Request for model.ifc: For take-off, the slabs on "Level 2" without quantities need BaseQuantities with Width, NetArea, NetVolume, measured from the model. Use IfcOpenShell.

First a look at what the model holds.

```python
import ifcopenshell
import ifcopenshell.util.element
import ifcopenshell.util.unit

model = ifcopenshell.open("model.ifc")
print(model.schema)
for unit_type in ("LENGTHUNIT", "AREAUNIT", "VOLUMEUNIT"):
    print(unit_type, ifcopenshell.util.unit.calculate_unit_scale(model, unit_type))
storey = next(s for s in model.by_type("IfcBuildingStorey") if s.Name == "Level 2")
slabs = [e for e in ifcopenshell.util.element.get_decomposition(storey) if e.is_a("IfcSlab")]
for e in sorted(slabs, key=lambda e: e.id()):
    print(e.id(), e.is_a(), e.Name, list(ifcopenshell.util.element.get_psets(e, qtos_only=True)), sep=" | ")
```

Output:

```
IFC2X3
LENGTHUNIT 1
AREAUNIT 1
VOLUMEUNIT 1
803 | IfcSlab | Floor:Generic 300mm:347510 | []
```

```python
import ifcopenshell
import ifcopenshell.api.pset
import ifcopenshell.geom
import ifcopenshell.util.element
import ifcopenshell.util.shape
import ifcopenshell.util.unit

model = ifcopenshell.open("model.ifc")
unit_scale = ifcopenshell.util.unit.calculate_unit_scale(model)
area_scale = ifcopenshell.util.unit.calculate_unit_scale(model, "AREAUNIT")
volume_scale = ifcopenshell.util.unit.calculate_unit_scale(model, "VOLUMEUNIT")
settings = ifcopenshell.geom.settings()

storey = next(s for s in model.by_type("IfcBuildingStorey") if s.Name == "Level 2")
slabs = [e for e in ifcopenshell.util.element.get_decomposition(storey) if e.is_a("IfcSlab")]

for e in sorted(slabs, key=lambda e: e.id()):
    if ifcopenshell.util.element.get_psets(e, qtos_only=True, should_inherit=False):
        continue
    # Geometry comes back in metres, in the element's own axes.
    shape = ifcopenshell.geom.create_shape(settings, e)
    values = {
        "Width": ifcopenshell.util.shape.get_z(shape.geometry) / unit_scale,
        "NetArea": ifcopenshell.util.shape.get_footprint_area(shape.geometry) / area_scale,
        "NetVolume": ifcopenshell.util.shape.get_volume(shape.geometry) / volume_scale,
    }
    qto = ifcopenshell.api.pset.add_qto(model, product=e, name="BaseQuantities")
    ifcopenshell.api.pset.edit_qto(model, qto=qto, properties=values)
    print(e.id(), {k: round(v, 3) for k, v in values.items()})

model.write("model_updated.ifc")
```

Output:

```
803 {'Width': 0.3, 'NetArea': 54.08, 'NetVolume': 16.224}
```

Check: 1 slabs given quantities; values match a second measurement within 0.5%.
